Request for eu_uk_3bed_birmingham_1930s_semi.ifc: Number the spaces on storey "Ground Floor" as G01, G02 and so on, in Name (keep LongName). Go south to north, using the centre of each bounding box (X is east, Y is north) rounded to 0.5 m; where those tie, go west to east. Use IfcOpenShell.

First a look at what the model holds.

```python
import ifcopenshell
import ifcopenshell.util.element
import ifcopenshell.util.placement

model = ifcopenshell.open("eu_uk_3bed_birmingham_1930s_semi.ifc")
print(model.schema)
storey = next(s for s in model.by_type("IfcBuildingStorey") if s.Name == "Ground Floor")
spaces = [e for e in ifcopenshell.util.element.get_decomposition(storey) if e.is_a("IfcSpace")]
for e in sorted(spaces, key=lambda e: e.id()):
    origin = ifcopenshell.util.placement.get_local_placement(e.ObjectPlacement)[:3, 3]
    print(e.id(), e.Name, e.LongName, origin.round(2) + 0.0, sep=" | ")
```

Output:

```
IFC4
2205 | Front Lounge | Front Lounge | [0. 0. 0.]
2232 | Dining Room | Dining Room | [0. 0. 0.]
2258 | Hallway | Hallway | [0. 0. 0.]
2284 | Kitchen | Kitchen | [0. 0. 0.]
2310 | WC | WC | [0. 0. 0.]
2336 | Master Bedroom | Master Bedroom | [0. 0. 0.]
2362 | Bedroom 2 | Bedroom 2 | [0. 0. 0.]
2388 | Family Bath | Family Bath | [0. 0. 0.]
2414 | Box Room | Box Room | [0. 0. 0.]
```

```python
import ifcopenshell
import ifcopenshell.geom
import ifcopenshell.util.element
import ifcopenshell.util.shape

model = ifcopenshell.open("eu_uk_3bed_birmingham_1930s_semi.ifc")
settings = ifcopenshell.geom.settings()
settings.set("use-world-coords", True)


def centre(element):
    shape = ifcopenshell.geom.create_shape(settings, element)
    return ifcopenshell.util.shape.get_bbox_centroid(shape.geometry)


storey = next(s for s in model.by_type("IfcBuildingStorey") if s.Name == "Ground Floor")
spaces = [e for e in ifcopenshell.util.element.get_decomposition(storey) if e.is_a("IfcSpace")]

# Insertion points can sit at a corner or the storey origin, so sort by the geometry (in metres).
centres = {e: centre(e) for e in spaces}
spaces.sort(key=lambda e: (round(centres[e][1] / 0.5), centres[e][0]))

for i, e in enumerate(spaces, start=1):
    number = f"G{i:02d}"
    e.Name = number
    print(e.id(), number)

model.write("eu_uk_3bed_birmingham_1930s_semi-out.ifc")
```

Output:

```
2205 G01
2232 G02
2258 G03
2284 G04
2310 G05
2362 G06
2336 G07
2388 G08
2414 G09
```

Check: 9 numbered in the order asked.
